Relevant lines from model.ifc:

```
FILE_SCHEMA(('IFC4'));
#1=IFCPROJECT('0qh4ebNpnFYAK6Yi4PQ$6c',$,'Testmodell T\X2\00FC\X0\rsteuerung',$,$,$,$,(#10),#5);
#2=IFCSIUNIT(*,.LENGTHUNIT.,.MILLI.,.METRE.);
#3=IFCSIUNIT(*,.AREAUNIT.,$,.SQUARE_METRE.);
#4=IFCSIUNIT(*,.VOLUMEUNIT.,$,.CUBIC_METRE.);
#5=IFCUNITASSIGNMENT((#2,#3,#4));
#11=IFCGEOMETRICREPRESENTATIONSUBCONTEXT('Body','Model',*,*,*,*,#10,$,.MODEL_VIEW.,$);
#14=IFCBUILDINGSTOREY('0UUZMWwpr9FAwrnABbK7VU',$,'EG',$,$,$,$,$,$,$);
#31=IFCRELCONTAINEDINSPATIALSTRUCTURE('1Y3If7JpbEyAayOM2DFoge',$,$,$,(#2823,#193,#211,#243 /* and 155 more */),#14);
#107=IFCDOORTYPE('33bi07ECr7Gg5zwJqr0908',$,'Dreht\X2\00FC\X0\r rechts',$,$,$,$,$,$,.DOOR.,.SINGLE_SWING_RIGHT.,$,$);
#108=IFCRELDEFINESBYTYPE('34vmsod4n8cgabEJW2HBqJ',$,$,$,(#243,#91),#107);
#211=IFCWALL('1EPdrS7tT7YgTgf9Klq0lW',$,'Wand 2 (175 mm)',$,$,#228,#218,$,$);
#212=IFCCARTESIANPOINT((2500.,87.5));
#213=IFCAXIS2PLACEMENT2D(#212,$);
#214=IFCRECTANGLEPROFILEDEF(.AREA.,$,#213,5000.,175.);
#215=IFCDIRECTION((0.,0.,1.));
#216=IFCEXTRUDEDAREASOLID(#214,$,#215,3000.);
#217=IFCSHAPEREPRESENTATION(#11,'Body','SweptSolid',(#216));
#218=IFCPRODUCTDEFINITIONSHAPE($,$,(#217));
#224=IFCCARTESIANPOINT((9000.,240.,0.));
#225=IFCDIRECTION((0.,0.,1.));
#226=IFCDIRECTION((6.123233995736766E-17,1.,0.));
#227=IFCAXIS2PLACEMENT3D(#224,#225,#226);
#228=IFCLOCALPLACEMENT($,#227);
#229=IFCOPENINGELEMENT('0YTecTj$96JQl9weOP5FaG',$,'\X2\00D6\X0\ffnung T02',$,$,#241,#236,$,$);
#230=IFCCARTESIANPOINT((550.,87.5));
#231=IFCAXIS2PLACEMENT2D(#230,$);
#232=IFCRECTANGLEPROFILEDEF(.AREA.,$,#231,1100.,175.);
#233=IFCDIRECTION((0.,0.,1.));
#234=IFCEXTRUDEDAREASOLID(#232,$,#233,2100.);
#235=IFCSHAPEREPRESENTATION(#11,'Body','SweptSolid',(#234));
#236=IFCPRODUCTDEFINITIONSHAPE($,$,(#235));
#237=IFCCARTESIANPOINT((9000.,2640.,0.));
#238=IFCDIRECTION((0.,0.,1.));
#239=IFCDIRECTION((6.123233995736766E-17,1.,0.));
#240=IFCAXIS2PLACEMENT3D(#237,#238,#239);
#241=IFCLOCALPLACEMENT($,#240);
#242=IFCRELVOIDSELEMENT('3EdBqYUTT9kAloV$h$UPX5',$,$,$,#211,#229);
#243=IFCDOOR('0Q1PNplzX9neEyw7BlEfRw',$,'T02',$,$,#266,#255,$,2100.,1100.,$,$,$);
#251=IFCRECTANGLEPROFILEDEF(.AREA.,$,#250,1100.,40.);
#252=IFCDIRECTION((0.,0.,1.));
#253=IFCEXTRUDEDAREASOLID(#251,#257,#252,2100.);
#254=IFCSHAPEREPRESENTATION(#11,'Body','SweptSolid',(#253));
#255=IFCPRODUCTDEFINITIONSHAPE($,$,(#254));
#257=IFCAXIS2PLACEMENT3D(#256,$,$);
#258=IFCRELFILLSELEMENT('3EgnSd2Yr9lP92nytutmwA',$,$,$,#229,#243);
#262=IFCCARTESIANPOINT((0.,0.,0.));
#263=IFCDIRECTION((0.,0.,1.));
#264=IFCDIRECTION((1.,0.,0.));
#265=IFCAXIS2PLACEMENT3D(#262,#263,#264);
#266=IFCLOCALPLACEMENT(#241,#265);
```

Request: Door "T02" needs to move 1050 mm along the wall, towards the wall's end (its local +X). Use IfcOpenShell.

```python
import ifcopenshell
import ifcopenshell.api.geometry
import ifcopenshell.util.placement

model = ifcopenshell.open("model.ifc")

door = model.by_guid("0Q1PNplzX9neEyw7BlEfRw")
opening = door.FillsVoids[0].RelatingOpeningElement
wall = opening.VoidsElements[0].RelatingBuildingElement

wall_matrix = ifcopenshell.util.placement.get_local_placement(wall.ObjectPlacement)
shift = wall_matrix[:3, 0] * 1050.0
before = ifcopenshell.util.placement.get_local_placement(door.ObjectPlacement)[:3, 3].copy()

# The door is placed relative to its opening, so it follows when the opening moves.
matrix = ifcopenshell.util.placement.get_local_placement(opening.ObjectPlacement)
matrix[:3, 3] += shift
ifcopenshell.api.geometry.edit_object_placement(
    model, product=opening, matrix=matrix, is_si=False, should_transform_children=True
)

after = ifcopenshell.util.placement.get_local_placement(door.ObjectPlacement)[:3, 3]
print("door moved by", (after - before).round(3) + 0.0)

model.write("model_edited.ifc")
```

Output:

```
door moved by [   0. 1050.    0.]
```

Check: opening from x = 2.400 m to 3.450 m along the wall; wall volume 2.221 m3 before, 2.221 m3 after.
